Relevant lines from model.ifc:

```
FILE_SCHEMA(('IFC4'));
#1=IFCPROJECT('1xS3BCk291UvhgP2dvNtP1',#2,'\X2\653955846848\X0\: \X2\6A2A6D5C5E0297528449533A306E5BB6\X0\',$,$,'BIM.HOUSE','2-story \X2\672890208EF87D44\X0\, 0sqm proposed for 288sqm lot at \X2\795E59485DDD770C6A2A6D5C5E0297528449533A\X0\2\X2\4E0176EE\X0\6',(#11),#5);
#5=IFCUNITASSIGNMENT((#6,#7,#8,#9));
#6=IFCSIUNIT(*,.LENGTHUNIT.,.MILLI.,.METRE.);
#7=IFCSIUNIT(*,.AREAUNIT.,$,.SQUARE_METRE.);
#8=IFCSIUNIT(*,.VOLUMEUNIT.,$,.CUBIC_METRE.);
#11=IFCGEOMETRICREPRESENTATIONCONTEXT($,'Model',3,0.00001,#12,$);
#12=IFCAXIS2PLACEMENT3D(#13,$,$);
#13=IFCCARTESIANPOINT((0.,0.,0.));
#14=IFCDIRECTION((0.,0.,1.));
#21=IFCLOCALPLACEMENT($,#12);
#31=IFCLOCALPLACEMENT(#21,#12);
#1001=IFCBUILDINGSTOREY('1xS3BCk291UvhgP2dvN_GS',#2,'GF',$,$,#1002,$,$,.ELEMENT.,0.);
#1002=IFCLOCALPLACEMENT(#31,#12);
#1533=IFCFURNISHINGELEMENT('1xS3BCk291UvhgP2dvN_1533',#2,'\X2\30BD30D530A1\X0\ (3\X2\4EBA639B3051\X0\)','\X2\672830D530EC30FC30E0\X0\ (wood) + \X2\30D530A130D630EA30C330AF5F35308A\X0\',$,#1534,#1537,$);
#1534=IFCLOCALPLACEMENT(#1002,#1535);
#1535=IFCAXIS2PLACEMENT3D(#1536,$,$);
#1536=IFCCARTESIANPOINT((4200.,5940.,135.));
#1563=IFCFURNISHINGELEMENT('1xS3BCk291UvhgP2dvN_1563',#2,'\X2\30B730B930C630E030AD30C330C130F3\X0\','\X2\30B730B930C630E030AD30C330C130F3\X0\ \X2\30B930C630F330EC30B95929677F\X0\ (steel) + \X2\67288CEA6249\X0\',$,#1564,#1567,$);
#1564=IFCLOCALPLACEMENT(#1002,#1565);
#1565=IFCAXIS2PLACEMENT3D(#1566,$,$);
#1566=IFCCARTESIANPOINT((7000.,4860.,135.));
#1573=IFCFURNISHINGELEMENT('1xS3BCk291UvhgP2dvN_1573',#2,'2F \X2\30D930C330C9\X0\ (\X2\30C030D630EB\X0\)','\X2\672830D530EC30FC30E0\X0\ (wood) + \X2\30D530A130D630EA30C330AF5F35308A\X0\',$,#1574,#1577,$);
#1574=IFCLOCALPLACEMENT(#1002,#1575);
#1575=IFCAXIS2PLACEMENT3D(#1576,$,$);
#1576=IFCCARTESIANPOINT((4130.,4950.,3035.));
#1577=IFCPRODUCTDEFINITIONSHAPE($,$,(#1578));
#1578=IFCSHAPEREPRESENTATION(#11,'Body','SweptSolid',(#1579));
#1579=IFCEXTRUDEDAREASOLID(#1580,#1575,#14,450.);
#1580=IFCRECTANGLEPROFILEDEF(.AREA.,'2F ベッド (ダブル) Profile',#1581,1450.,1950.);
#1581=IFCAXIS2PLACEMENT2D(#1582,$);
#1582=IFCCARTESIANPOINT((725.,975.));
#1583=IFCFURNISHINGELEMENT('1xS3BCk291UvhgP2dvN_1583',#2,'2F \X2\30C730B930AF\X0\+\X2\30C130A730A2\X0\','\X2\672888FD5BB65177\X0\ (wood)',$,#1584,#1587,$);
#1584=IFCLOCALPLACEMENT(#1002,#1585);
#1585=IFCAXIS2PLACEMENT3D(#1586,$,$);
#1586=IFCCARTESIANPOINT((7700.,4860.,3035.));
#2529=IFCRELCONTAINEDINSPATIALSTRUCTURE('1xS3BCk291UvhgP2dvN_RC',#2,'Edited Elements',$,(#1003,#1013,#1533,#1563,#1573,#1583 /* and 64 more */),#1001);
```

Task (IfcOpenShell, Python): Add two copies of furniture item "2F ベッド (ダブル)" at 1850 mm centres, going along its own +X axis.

```python
import ifcopenshell
import ifcopenshell.api.geometry
import ifcopenshell.api.root
import ifcopenshell.util.element
import ifcopenshell.util.placement

model = ifcopenshell.open("model.ifc")


def reuse_history(source, copy):
    """copy_class also copies each property set's owner history, people and application; keep the originals."""
    for rel in copy.IsDefinedBy:
        if rel.is_a("IfcRelDefinesByProperties") and (history := rel.RelatingPropertyDefinition.OwnerHistory):
            rel.RelatingPropertyDefinition.OwnerHistory = source.OwnerHistory
            ifcopenshell.util.element.remove_deep2(model, history)


source = model.by_id(1573)
base = ifcopenshell.util.placement.get_local_placement(source.ObjectPlacement)
step = base[:3, 0] * 1850.0

for i in range(1, 3):
    copy = ifcopenshell.api.root.copy_class(model, product=source)
    copy.Representation = ifcopenshell.util.element.copy_deep(
        model, source.Representation, exclude=["IfcGeometricRepresentationContext", "IfcRepresentationMap"]
    )
    reuse_history(source, copy)
    matrix = base.copy()
    matrix[:3, 3] += i * step
    print("added at", matrix[:3, 3].round(3) + 0.0)
    ifcopenshell.api.geometry.edit_object_placement(model, product=copy, matrix=matrix, is_si=False)

model.write("model_edited.ifc")
```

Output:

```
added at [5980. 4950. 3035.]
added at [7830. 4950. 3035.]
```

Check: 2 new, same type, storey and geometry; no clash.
